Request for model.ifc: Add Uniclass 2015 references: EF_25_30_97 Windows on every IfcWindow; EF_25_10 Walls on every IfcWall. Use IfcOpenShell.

First a look at what the model holds.

```python
import ifcopenshell

model = ifcopenshell.open("model.ifc")
print(model.schema)
print("classifications:", [c.Name for c in model.by_type("IfcClassification")])
for ifc_class in ("IfcDoor", "IfcRoof", "IfcStair", "IfcWall", "IfcWindow"):
    print(ifc_class, len(model.by_type(ifc_class)))
```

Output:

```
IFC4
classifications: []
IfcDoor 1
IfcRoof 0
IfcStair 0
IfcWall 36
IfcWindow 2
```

```python
import ifcopenshell
import ifcopenshell.api.classification

model = ifcopenshell.open("model.ifc")

system = ifcopenshell.api.classification.add_classification(model, classification="Uniclass 2015")

codes = {
    "IfcWindow": ("EF_25_30_97", "Windows"),
    "IfcWall": ("EF_25_10", "Walls"),
}
for ifc_class, (code, name) in codes.items():
    products = model.by_type(ifc_class)
    ifcopenshell.api.classification.add_reference(
        model, products=products, classification=system, identification=code, name=name
    )
    print(code, len(products))

model.write("model_rev.ifc")
```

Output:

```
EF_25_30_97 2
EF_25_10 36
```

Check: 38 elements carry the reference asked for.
